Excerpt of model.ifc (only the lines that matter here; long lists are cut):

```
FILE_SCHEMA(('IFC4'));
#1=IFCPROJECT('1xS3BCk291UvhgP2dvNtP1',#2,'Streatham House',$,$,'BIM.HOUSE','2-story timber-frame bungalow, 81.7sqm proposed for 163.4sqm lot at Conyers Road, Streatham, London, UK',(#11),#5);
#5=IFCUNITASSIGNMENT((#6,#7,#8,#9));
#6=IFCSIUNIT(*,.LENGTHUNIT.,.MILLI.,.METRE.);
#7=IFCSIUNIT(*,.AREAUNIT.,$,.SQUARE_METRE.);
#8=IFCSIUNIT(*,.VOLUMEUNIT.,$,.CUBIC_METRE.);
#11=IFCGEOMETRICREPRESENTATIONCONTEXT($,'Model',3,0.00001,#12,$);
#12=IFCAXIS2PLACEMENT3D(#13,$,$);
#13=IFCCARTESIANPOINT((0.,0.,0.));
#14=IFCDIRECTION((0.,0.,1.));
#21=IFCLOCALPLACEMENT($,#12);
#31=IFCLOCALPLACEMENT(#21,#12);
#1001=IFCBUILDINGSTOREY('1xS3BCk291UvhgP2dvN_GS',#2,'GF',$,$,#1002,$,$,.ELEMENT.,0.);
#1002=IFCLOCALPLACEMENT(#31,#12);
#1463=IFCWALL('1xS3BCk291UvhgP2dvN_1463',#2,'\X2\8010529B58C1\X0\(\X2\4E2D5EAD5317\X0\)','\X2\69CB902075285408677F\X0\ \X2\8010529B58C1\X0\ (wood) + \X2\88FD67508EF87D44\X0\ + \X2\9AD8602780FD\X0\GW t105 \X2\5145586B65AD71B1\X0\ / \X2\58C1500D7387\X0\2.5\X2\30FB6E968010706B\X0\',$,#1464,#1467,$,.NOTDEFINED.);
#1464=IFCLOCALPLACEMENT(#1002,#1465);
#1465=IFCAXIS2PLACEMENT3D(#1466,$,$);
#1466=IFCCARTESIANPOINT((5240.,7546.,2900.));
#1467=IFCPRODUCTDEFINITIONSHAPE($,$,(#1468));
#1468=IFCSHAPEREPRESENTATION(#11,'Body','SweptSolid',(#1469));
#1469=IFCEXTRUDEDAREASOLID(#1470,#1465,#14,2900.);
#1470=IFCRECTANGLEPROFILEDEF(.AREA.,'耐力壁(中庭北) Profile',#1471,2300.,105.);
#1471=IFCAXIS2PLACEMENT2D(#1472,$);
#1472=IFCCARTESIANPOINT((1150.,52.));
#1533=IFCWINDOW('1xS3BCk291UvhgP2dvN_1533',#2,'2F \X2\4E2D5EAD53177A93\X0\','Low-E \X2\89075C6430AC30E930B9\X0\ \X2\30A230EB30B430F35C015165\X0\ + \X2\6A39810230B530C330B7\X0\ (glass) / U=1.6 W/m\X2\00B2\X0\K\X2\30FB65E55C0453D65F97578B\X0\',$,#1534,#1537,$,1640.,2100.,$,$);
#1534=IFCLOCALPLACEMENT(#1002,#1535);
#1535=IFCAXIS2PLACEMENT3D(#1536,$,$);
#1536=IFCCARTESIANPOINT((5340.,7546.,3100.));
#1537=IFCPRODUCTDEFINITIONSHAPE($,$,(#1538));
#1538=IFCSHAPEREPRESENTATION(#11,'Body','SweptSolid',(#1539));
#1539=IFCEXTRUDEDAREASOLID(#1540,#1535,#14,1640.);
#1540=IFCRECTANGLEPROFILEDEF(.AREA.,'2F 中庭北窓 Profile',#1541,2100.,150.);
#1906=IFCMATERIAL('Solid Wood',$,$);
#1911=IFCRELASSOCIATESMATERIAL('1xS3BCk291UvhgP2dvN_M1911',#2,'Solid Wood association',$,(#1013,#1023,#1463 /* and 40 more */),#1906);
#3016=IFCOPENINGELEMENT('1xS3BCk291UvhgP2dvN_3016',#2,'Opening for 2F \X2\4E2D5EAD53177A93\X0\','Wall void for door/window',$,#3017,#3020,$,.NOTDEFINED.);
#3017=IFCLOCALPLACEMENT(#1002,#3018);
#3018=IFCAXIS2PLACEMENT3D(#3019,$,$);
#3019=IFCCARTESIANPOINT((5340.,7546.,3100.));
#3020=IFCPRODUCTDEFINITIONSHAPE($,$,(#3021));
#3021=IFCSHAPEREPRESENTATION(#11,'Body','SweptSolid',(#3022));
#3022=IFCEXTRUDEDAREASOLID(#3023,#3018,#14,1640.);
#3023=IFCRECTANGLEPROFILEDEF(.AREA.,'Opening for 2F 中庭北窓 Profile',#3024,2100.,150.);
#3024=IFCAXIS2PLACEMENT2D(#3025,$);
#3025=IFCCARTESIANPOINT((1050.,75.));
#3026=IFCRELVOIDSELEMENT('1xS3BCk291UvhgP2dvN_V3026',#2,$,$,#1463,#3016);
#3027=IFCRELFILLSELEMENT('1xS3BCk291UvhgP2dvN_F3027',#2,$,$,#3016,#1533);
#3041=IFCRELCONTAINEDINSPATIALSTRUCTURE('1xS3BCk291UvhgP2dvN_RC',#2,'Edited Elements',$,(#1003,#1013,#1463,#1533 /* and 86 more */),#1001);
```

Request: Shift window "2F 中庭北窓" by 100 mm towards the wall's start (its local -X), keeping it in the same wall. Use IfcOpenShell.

```python
import ifcopenshell
import ifcopenshell.api.geometry
import ifcopenshell.util.placement
import ifcopenshell.util.unit

model = ifcopenshell.open("model.ifc")
unit_scale = ifcopenshell.util.unit.calculate_unit_scale(model)

window = model.by_guid("1xS3BCk291UvhgP2dvN_1533")
opening = window.FillsVoids[0].RelatingOpeningElement
wall = opening.VoidsElements[0].RelatingBuildingElement

wall_matrix = ifcopenshell.util.placement.get_local_placement(wall.ObjectPlacement)
shift = wall_matrix[:3, 0] * -0.1 / unit_scale
before = ifcopenshell.util.placement.get_local_placement(window.ObjectPlacement)[:3, 3].copy()

# The window is not placed relative to its opening, so move both.
for product in (opening, window):
    matrix = ifcopenshell.util.placement.get_local_placement(product.ObjectPlacement)
    matrix[:3, 3] += shift
    ifcopenshell.api.geometry.edit_object_placement(model, product=product, matrix=matrix, is_si=False)

after = ifcopenshell.util.placement.get_local_placement(window.ObjectPlacement)[:3, 3]
print("window moved by", (after - before).round(3) + 0.0)

model.write("model_v2.ifc")
```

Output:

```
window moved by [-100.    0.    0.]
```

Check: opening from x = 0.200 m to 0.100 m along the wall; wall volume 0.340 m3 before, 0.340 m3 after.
